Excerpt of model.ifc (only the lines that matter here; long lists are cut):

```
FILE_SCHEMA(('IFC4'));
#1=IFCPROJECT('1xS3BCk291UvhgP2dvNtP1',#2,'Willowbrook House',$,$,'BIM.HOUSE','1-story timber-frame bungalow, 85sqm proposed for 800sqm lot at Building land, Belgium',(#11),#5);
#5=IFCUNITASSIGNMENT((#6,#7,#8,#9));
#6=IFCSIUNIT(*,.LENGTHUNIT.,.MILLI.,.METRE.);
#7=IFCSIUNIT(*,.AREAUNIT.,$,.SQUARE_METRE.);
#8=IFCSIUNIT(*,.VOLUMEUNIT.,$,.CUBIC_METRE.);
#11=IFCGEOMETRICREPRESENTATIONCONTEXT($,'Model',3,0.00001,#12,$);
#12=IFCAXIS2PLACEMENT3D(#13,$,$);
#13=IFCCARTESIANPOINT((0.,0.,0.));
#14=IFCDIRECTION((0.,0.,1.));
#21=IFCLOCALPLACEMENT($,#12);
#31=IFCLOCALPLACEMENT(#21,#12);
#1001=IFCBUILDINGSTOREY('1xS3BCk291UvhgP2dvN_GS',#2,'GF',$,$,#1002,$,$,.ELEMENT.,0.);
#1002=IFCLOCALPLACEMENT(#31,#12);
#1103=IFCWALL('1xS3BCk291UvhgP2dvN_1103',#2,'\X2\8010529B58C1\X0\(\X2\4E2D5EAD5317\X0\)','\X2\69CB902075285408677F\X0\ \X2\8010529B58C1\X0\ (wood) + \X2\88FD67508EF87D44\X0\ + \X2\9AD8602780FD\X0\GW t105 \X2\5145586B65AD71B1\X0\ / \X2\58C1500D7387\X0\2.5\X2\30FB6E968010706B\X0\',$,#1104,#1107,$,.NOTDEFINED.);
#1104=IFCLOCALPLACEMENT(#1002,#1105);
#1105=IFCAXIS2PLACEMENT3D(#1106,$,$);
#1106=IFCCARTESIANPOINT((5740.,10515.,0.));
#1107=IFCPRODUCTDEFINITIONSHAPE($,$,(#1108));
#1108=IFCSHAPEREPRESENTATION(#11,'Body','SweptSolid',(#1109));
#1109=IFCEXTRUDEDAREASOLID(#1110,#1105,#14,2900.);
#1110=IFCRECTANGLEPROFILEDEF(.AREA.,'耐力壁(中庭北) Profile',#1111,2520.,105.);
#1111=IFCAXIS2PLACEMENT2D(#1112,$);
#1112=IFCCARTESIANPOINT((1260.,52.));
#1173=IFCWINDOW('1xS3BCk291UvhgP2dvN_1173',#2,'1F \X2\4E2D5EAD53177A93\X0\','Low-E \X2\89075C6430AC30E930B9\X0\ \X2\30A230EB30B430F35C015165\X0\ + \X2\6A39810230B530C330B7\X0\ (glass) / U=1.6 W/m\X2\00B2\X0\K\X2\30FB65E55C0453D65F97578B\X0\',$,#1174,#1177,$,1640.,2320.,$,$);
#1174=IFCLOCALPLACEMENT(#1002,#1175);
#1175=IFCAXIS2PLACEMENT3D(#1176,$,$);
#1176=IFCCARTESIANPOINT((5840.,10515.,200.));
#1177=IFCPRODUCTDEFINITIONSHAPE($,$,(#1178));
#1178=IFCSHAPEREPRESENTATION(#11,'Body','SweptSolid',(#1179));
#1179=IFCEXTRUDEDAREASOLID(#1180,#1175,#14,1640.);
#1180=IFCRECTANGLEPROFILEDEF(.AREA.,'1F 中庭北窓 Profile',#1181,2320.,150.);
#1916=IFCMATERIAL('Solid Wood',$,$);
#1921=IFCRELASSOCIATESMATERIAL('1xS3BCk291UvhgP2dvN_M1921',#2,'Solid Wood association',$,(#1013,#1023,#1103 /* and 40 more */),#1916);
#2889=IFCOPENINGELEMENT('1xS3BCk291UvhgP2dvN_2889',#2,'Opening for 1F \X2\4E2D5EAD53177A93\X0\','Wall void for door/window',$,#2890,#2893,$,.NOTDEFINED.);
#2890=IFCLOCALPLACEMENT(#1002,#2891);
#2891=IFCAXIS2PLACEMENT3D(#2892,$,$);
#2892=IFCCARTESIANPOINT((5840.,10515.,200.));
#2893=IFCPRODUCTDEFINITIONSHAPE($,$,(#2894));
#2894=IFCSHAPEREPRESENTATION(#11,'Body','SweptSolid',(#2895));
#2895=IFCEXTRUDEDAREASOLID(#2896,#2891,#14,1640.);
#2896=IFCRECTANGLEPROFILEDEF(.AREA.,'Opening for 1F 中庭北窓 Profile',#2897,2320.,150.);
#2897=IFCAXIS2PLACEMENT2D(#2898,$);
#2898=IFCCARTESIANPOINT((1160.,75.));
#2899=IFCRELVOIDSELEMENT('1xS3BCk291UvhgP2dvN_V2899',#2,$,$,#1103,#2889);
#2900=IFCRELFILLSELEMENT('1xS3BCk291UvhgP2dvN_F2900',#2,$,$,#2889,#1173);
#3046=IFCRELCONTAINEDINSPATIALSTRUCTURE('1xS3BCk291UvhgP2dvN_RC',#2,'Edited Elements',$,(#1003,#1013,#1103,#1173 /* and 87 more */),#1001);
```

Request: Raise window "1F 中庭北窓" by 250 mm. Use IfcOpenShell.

```python
import numpy as np
import ifcopenshell
import ifcopenshell.api.geometry
import ifcopenshell.util.placement
import ifcopenshell.util.unit

model = ifcopenshell.open("model.ifc")
unit_scale = ifcopenshell.util.unit.calculate_unit_scale(model)

window = model.by_guid("1xS3BCk291UvhgP2dvN_1173")
opening = window.FillsVoids[0].RelatingOpeningElement
dz = 0.25 / unit_scale

shift = np.array([0.0, 0.0, dz])
# The window is not placed relative to its opening, so move both.
for product in (opening, window):
    matrix = ifcopenshell.util.placement.get_local_placement(product.ObjectPlacement)
    matrix[:3, 3] += shift
    ifcopenshell.api.geometry.edit_object_placement(model, product=product, matrix=matrix, is_si=False)

print(f"moved by {dz * unit_scale:+.3f} m")

model.write("model_v2.ifc")
```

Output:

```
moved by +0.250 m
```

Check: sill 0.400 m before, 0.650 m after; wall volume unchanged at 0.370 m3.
